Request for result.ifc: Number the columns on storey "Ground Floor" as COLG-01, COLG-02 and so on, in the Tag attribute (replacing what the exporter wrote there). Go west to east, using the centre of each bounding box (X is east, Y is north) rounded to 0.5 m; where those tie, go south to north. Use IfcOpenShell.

First a look at what the model holds.

```python
import ifcopenshell
import ifcopenshell.util.element
import ifcopenshell.util.placement

model = ifcopenshell.open("result.ifc")
print(model.schema)
storey = next(s for s in model.by_type("IfcBuildingStorey") if s.Name == "Ground Floor")
columns = [e for e in ifcopenshell.util.element.get_decomposition(storey) if e.is_a("IfcColumn")]
for e in sorted(columns, key=lambda e: e.id()):
    origin = ifcopenshell.util.placement.get_local_placement(e.ObjectPlacement)[:3, 3]
    print(e.id(), e.Tag, e.Name, origin.round(2) + 0.0, sep=" | ")
```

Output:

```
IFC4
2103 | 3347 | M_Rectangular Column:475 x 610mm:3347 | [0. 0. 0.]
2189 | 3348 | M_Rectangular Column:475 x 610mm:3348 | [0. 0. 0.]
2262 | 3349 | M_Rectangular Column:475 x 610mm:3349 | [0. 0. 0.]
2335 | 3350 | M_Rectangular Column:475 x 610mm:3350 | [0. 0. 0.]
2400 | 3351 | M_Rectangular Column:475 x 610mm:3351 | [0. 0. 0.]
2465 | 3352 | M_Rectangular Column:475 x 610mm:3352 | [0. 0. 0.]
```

```python
import ifcopenshell
import ifcopenshell.geom
import ifcopenshell.util.element
import ifcopenshell.util.shape

model = ifcopenshell.open("result.ifc")
settings = ifcopenshell.geom.settings()
settings.set("use-world-coords", True)


def centre(element):
    shape = ifcopenshell.geom.create_shape(settings, element)
    return ifcopenshell.util.shape.get_bbox_centroid(shape.geometry)


storey = next(s for s in model.by_type("IfcBuildingStorey") if s.Name == "Ground Floor")
columns = [e for e in ifcopenshell.util.element.get_decomposition(storey) if e.is_a("IfcColumn")]

# Insertion points can sit at a corner or the storey origin, so sort by the geometry (in metres).
centres = {e: centre(e) for e in columns}
columns.sort(key=lambda e: (round(centres[e][0] / 0.5), centres[e][1]))

for i, e in enumerate(columns, start=1):
    number = f"COLG-{i:02d}"
    e.Tag = number
    print(e.id(), number)

model.write("result_rev.ifc")
```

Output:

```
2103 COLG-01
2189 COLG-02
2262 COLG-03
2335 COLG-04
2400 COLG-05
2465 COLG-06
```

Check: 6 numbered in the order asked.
